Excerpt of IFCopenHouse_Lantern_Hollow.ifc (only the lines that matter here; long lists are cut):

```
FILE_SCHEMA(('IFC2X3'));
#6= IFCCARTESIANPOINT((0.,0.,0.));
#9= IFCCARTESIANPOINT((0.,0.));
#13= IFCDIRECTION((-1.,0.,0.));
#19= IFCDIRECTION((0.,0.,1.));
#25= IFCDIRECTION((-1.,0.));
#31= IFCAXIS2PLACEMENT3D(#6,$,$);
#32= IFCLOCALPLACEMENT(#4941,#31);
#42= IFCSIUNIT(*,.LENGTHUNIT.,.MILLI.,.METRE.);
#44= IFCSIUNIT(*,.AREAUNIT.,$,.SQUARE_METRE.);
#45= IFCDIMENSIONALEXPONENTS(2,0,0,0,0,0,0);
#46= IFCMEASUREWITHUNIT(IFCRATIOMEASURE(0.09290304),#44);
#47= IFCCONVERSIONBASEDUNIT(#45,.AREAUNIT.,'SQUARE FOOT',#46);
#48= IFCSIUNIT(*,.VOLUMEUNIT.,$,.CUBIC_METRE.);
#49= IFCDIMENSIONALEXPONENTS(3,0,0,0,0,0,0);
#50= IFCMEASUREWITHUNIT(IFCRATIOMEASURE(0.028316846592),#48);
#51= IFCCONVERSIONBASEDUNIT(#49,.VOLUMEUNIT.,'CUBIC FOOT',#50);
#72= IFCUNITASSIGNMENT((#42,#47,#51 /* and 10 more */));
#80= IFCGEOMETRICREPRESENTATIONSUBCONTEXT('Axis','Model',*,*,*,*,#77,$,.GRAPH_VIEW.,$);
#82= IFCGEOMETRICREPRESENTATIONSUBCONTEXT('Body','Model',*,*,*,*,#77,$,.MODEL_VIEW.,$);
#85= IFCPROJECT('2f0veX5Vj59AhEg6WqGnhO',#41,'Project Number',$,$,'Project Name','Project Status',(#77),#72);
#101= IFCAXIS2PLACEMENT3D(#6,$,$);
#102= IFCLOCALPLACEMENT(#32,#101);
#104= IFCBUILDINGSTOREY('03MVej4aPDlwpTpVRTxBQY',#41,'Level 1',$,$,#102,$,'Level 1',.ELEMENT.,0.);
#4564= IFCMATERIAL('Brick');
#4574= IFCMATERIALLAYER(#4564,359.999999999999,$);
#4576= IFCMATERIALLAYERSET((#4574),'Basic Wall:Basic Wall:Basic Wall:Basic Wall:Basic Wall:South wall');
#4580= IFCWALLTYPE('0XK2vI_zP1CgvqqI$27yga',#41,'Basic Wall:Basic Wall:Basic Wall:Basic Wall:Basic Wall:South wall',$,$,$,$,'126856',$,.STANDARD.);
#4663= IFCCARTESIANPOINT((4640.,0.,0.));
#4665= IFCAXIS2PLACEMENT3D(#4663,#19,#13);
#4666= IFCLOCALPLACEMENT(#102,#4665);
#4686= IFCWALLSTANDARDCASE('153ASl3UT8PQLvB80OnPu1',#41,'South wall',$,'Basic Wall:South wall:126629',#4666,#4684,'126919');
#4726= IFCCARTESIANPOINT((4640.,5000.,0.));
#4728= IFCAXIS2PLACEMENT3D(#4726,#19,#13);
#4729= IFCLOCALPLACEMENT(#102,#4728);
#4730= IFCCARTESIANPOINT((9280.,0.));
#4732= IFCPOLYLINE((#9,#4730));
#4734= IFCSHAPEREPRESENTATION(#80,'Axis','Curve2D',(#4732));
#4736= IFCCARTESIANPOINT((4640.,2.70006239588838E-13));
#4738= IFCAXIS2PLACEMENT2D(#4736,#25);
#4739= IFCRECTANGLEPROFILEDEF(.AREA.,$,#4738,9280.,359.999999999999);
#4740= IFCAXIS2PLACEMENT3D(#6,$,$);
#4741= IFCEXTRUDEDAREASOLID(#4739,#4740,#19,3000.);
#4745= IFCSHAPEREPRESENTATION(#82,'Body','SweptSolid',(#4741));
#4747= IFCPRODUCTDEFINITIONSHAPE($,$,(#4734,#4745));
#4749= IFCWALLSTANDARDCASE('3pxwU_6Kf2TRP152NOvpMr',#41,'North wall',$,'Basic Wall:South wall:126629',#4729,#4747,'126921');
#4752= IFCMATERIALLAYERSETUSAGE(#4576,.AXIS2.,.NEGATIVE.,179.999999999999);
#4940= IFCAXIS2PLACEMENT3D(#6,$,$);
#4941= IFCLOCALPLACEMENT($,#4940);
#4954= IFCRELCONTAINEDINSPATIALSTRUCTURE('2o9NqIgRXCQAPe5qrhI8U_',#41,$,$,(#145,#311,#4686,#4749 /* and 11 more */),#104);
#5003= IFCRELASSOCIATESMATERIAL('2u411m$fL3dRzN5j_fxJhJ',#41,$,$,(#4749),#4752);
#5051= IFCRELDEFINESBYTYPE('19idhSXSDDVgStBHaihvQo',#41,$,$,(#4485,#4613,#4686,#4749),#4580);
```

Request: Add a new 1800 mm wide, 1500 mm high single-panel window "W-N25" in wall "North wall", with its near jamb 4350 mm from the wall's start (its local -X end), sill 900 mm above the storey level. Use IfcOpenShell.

```python
import numpy as np
import ifcopenshell
import ifcopenshell.api.feature
import ifcopenshell.api.geometry
import ifcopenshell.api.root
import ifcopenshell.api.spatial
import ifcopenshell.api.type
import ifcopenshell.geom
import ifcopenshell.util.element
import ifcopenshell.util.placement
import ifcopenshell.util.representation
import ifcopenshell.util.shape
import ifcopenshell.util.unit

model = ifcopenshell.open("IFCopenHouse_Lantern_Hollow.ifc")
unit_scale = ifcopenshell.util.unit.calculate_unit_scale(model)
settings = ifcopenshell.geom.settings()


def volume(element):
    """Net volume in cubic metres, openings subtracted."""
    shape = ifcopenshell.geom.create_shape(settings, element)
    return ifcopenshell.util.shape.get_volume(shape.geometry)


wall = model.by_id(4749)
storey = ifcopenshell.util.element.get_container(wall, ifc_class="IfcBuildingStorey")
context = ifcopenshell.util.representation.get_context(model, "Model", "Body", "MODEL_VIEW")
before = volume(wall)

width, height, from_end, sill = 1.8, 1.5, 4.35, 0.9  # metres

# The wall runs along its own X axis, and the end named is its -X end.
wall_shape = ifcopenshell.geom.create_shape(settings, wall)
x, y, z = ifcopenshell.util.shape.get_vertices(wall_shape.geometry).T
start = x.min() + from_end
face, thickness = float(y.min()), float(y.max() - y.min())
wall_matrix = ifcopenshell.util.placement.get_local_placement(wall.ObjectPlacement)
level = ifcopenshell.util.placement.get_local_placement(storey.ObjectPlacement)[2, 3]


def in_wall(x, y):
    """Placement at x, y metres in the wall's axes, at sill height."""
    matrix = wall_matrix.copy()
    matrix[:, 3] = wall_matrix @ np.array([x / unit_scale, y / unit_scale, 0.0, 1.0])
    matrix[2, 3] = level + sill / unit_scale
    return matrix


# Opening: a box that overshoots both wall faces by 50 mm.
opening = ifcopenshell.api.root.create_entity(model, ifc_class="IfcOpeningElement")
box = ifcopenshell.api.geometry.add_wall_representation(
    model, context=context, length=width, height=height, thickness=thickness + 0.1
)
ifcopenshell.api.geometry.assign_representation(model, product=opening, representation=box)
ifcopenshell.api.geometry.edit_object_placement(model, product=opening, matrix=in_wall(start, face - 0.05), is_si=False)
ifcopenshell.api.feature.add_feature(model, feature=opening, element=wall)

window = ifcopenshell.api.root.create_entity(model, ifc_class="IfcWindow", name="W-N25")
window.OverallWidth, window.OverallHeight = width / unit_scale, height / unit_scale
body = ifcopenshell.api.geometry.add_window_representation(
    model,
    context=context,
    overall_width=window.OverallWidth,
    overall_height=window.OverallHeight,
    partition_type="SINGLE_PANEL",
)
ifcopenshell.api.geometry.assign_representation(model, product=window, representation=body)
ifcopenshell.api.spatial.assign_container(model, products=[window], relating_structure=storey)
fills = ifcopenshell.api.feature.add_filling(model, opening=opening, element=window)
fills.OwnerHistory = window.OwnerHistory  # required in IFC2X3

# IFC2X3 keeps the operation on the window style.
style = ifcopenshell.api.root.create_entity(model, ifc_class="IfcWindowStyle", name="W-N25")
style.OperationType, style.ConstructionType = "SINGLE_PANEL", "NOTDEFINED"
style.ParameterTakesPrecedence = style.Sizeable = False
ifcopenshell.api.type.assign_type(model, related_objects=[window], relating_type=style)

# Centre the window in the wall's thickness.
ifcopenshell.api.geometry.edit_object_placement(model, product=window, matrix=in_wall(start, face), is_si=False)
window_shape = ifcopenshell.geom.create_shape(settings, window)
depth = ifcopenshell.util.shape.get_vertices(window_shape.geometry)[:, 1]
offset = face + thickness / 2 - (depth.min() + depth.max()) / 2
ifcopenshell.api.geometry.edit_object_placement(model, product=window, matrix=in_wall(start, offset), is_si=False)

after = volume(wall)

print(f"wall volume {before:.3f} -> {after:.3f} m3")

model.write("IFCopenHouse_Lantern_Hollow_v2.ifc")
```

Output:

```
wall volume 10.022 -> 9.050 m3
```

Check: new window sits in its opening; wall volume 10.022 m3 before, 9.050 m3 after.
